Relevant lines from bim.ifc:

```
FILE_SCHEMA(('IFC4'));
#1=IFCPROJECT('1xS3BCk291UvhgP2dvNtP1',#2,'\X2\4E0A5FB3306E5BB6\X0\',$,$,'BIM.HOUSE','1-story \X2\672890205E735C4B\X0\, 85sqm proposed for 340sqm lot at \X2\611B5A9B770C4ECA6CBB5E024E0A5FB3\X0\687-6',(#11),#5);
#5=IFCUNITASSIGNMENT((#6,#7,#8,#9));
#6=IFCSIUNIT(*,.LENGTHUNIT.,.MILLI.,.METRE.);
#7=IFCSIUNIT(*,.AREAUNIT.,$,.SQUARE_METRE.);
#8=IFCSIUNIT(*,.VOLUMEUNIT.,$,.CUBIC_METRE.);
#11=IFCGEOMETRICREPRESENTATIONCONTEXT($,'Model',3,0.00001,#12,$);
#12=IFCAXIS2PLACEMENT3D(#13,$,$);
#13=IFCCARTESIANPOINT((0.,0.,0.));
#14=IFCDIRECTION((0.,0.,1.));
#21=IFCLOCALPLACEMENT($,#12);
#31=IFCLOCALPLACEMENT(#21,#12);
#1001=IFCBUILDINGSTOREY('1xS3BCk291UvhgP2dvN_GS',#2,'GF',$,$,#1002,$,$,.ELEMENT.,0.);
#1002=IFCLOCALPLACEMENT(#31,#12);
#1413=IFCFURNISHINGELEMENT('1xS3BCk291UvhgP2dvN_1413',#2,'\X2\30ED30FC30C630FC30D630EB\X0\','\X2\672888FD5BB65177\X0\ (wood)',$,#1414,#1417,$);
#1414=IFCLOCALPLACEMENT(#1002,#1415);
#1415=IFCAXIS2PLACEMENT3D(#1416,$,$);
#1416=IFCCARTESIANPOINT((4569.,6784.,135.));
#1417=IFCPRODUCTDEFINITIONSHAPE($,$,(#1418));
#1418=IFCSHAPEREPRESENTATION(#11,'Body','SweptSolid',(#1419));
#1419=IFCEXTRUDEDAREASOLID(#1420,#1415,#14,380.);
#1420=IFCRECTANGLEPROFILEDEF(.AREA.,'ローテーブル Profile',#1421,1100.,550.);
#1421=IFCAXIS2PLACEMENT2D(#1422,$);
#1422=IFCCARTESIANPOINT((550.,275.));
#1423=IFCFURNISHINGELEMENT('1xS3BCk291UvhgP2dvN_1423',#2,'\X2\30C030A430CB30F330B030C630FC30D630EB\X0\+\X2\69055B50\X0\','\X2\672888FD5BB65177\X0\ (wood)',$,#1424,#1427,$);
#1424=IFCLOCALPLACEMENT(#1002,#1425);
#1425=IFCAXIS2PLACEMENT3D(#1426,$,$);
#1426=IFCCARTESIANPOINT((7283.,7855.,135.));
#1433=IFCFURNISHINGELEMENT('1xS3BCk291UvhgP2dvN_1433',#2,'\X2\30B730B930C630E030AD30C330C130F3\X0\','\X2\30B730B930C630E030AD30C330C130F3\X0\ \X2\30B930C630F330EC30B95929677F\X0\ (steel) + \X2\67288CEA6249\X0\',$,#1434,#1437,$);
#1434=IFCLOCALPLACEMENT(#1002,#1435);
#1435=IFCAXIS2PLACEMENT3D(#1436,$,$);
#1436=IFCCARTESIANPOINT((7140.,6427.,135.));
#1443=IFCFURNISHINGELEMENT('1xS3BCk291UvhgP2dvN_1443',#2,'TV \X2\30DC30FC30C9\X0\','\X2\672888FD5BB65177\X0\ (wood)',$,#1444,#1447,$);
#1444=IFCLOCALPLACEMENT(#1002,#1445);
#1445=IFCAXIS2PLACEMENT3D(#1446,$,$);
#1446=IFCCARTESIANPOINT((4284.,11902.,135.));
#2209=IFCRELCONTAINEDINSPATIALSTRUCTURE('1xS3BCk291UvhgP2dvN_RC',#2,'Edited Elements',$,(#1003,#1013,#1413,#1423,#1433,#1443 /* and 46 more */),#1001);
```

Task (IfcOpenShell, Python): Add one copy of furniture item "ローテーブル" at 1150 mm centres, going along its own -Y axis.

```python
import ifcopenshell
import ifcopenshell.api.geometry
import ifcopenshell.api.root
import ifcopenshell.util.element
import ifcopenshell.util.placement
import ifcopenshell.util.unit

model = ifcopenshell.open("bim.ifc")
unit_scale = ifcopenshell.util.unit.calculate_unit_scale(model)


def reuse_history(source, copy):
    """copy_class also copies each property set's owner history, people and application; keep the originals."""
    for rel in copy.IsDefinedBy:
        if rel.is_a("IfcRelDefinesByProperties") and (history := rel.RelatingPropertyDefinition.OwnerHistory):
            rel.RelatingPropertyDefinition.OwnerHistory = source.OwnerHistory
            ifcopenshell.util.element.remove_deep2(model, history)


source = model.by_guid("1xS3BCk291UvhgP2dvN_1413")
base = ifcopenshell.util.placement.get_local_placement(source.ObjectPlacement)
step = -base[:3, 1] * 1.15 / unit_scale

for i in range(1, 2):
    copy = ifcopenshell.api.root.copy_class(model, product=source)
    copy.Representation = ifcopenshell.util.element.copy_deep(
        model, source.Representation, exclude=["IfcGeometricRepresentationContext", "IfcRepresentationMap"]
    )
    reuse_history(source, copy)
    matrix = base.copy()
    matrix[:3, 3] += i * step
    print("added at", matrix[:3, 3].round(3) + 0.0)
    ifcopenshell.api.geometry.edit_object_placement(model, product=copy, matrix=matrix, is_si=False)

model.write("bim_v2.ifc")
```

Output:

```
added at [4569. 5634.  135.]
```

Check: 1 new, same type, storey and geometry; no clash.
